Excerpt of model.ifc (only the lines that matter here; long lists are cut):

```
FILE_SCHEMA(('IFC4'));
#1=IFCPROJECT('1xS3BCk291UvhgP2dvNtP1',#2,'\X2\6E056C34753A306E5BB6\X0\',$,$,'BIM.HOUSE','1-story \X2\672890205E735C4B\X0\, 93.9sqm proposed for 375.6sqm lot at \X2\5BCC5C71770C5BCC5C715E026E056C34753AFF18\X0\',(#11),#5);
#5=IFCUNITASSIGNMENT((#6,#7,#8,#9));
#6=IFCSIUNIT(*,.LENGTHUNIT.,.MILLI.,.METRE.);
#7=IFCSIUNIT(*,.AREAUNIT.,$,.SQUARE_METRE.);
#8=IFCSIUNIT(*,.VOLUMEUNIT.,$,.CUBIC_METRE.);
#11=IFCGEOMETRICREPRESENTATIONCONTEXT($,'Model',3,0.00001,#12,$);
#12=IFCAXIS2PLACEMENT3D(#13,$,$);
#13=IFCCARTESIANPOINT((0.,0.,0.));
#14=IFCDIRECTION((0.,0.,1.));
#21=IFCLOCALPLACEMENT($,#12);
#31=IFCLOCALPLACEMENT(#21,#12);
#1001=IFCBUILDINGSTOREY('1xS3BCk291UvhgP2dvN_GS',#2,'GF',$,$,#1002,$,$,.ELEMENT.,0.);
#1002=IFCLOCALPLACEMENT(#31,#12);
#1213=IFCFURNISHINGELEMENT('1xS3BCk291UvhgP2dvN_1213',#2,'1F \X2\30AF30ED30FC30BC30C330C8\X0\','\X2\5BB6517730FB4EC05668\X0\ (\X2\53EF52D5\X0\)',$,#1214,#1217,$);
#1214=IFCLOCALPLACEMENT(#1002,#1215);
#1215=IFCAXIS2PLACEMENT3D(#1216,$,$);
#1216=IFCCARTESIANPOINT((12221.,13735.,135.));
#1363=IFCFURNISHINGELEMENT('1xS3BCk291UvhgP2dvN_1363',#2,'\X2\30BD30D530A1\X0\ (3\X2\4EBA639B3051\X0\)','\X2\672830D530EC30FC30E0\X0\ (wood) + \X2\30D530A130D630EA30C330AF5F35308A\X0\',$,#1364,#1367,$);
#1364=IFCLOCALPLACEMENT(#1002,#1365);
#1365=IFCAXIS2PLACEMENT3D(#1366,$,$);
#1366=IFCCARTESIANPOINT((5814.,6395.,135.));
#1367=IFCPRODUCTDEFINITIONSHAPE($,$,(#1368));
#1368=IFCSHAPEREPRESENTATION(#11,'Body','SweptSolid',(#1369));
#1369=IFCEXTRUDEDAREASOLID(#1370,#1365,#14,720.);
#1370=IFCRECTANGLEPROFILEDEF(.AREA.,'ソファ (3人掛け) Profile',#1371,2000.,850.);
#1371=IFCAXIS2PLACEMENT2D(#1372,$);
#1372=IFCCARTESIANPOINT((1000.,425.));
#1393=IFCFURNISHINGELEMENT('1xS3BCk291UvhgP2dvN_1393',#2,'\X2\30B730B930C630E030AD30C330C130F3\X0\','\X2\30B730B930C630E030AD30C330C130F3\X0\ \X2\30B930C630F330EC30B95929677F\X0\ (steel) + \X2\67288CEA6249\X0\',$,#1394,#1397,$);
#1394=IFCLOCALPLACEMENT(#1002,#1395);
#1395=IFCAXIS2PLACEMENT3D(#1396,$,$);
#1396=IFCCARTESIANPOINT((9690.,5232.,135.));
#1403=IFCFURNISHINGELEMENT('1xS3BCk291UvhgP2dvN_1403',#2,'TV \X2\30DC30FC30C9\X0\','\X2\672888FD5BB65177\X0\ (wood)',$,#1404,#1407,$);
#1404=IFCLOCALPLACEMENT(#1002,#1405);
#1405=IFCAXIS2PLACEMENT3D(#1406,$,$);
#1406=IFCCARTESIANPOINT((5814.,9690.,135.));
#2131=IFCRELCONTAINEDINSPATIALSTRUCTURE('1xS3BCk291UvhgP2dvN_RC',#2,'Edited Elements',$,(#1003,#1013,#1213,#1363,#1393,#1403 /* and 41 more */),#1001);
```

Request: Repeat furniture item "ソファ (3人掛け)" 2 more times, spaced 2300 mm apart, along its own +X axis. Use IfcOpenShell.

```python
import ifcopenshell
import ifcopenshell.api.geometry
import ifcopenshell.api.root
import ifcopenshell.util.element
import ifcopenshell.util.placement
import ifcopenshell.util.unit

model = ifcopenshell.open("model.ifc")
unit_scale = ifcopenshell.util.unit.calculate_unit_scale(model)


def reuse_history(source, copy):
    """copy_class also copies each property set's owner history, people and application; keep the originals."""
    for rel in copy.IsDefinedBy:
        if rel.is_a("IfcRelDefinesByProperties") and (history := rel.RelatingPropertyDefinition.OwnerHistory):
            rel.RelatingPropertyDefinition.OwnerHistory = source.OwnerHistory
            ifcopenshell.util.element.remove_deep2(model, history)


source = model.by_guid("1xS3BCk291UvhgP2dvN_1363")
base = ifcopenshell.util.placement.get_local_placement(source.ObjectPlacement)
step = base[:3, 0] * 2.3 / unit_scale

for i in range(1, 3):
    copy = ifcopenshell.api.root.copy_class(model, product=source)
    copy.Representation = ifcopenshell.util.element.copy_deep(
        model, source.Representation, exclude=["IfcGeometricRepresentationContext", "IfcRepresentationMap"]
    )
    reuse_history(source, copy)
    matrix = base.copy()
    matrix[:3, 3] += i * step
    print("added at", matrix[:3, 3].round(3) + 0.0)
    ifcopenshell.api.geometry.edit_object_placement(model, product=copy, matrix=matrix, is_si=False)

model.write("model-out.ifc")
```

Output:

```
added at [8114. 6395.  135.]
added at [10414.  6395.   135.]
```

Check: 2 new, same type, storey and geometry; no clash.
